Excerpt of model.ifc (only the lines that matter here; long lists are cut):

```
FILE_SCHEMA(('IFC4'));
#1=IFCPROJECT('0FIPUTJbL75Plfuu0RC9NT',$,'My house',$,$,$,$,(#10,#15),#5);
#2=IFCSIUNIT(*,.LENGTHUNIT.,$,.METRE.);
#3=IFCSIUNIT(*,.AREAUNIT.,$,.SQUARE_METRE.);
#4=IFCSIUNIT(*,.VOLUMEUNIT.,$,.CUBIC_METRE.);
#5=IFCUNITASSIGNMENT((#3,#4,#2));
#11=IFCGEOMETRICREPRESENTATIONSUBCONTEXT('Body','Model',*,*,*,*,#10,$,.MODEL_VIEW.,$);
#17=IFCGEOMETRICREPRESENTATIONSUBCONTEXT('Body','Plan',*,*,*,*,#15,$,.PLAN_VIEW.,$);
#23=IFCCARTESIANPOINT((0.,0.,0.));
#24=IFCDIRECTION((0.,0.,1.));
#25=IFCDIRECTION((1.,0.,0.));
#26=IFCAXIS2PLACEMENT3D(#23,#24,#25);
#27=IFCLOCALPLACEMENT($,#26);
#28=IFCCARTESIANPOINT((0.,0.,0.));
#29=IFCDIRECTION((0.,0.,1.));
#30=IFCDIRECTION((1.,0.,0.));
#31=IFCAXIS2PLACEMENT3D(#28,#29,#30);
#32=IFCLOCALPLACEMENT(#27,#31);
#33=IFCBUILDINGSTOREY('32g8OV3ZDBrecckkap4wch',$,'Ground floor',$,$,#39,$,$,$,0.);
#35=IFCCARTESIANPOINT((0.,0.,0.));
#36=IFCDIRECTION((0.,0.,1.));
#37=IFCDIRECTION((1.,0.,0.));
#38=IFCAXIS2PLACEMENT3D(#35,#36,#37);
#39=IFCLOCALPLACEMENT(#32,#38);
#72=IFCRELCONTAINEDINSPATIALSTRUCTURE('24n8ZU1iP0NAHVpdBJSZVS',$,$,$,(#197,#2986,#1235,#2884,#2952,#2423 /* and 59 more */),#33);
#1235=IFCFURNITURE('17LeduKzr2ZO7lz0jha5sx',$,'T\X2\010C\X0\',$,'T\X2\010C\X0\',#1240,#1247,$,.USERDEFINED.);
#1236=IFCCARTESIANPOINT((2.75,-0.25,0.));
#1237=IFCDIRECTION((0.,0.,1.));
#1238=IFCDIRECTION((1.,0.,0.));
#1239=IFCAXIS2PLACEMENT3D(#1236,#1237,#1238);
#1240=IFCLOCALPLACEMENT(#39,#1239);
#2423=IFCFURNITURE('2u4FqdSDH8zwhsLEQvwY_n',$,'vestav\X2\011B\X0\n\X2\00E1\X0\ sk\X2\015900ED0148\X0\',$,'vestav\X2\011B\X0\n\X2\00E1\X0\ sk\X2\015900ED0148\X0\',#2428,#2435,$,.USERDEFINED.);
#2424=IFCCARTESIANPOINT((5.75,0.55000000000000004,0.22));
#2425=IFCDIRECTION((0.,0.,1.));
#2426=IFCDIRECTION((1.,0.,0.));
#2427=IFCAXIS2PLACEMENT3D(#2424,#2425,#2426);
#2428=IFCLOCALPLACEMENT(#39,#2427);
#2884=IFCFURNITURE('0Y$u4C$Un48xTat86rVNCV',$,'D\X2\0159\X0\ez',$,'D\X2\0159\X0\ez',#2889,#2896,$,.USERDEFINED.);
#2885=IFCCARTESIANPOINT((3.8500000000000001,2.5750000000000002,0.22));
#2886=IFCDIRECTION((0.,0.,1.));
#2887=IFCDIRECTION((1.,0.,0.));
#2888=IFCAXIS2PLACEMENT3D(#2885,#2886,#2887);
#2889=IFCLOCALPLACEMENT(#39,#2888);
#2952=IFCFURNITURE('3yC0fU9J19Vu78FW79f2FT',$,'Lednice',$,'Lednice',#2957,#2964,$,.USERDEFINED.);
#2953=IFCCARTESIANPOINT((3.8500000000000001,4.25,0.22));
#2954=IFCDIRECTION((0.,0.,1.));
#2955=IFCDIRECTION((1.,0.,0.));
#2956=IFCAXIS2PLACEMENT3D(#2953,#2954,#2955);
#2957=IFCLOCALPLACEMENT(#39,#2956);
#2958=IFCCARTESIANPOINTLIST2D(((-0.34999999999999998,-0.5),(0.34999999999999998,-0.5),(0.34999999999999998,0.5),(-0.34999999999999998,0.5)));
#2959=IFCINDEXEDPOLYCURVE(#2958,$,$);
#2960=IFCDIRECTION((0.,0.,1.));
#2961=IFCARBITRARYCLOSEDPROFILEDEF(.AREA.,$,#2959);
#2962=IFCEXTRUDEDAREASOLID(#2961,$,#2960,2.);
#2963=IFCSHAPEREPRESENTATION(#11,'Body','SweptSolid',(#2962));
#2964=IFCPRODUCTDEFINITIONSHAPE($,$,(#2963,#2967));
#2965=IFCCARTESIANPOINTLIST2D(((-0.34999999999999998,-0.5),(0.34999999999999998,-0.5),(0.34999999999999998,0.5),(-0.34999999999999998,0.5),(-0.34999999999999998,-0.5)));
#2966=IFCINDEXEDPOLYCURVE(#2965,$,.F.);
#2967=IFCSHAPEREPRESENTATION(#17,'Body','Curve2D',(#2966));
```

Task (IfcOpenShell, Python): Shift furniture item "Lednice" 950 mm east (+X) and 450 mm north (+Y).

```python
import ifcopenshell
import ifcopenshell.api.geometry
import ifcopenshell.util.placement

model = ifcopenshell.open("model.ifc")

item = model.by_guid("3yC0fU9J19Vu78FW79f2FT")
matrix = ifcopenshell.util.placement.get_local_placement(item.ObjectPlacement)
matrix[0, 3] += 0.95
matrix[1, 3] += 0.45
ifcopenshell.api.geometry.edit_object_placement(model, product=item, matrix=matrix, is_si=False)

print(ifcopenshell.util.placement.get_local_placement(item.ObjectPlacement).round(3) + 0.0)

model.write("model-out.ifc")
```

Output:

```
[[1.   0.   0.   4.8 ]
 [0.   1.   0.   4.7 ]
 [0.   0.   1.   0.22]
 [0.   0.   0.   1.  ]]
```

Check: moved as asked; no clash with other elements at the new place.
